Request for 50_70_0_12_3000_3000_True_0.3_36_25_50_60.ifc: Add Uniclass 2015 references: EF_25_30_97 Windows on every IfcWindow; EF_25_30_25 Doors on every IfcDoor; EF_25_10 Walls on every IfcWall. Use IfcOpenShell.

First a look at what the model holds.

```python
import ifcopenshell

model = ifcopenshell.open("50_70_0_12_3000_3000_True_0.3_36_25_50_60.ifc")
print(model.schema)
print("classifications:", [c.Name for c in model.by_type("IfcClassification")])
for ifc_class in ("IfcDoor", "IfcRoof", "IfcStair", "IfcWall", "IfcWindow"):
    print(ifc_class, len(model.by_type(ifc_class)))
```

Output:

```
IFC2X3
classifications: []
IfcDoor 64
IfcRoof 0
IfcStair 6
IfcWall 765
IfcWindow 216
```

```python
import ifcopenshell
import ifcopenshell.api.classification

model = ifcopenshell.open("50_70_0_12_3000_3000_True_0.3_36_25_50_60.ifc")

# IFC2X3 requires Source and Edition and has no link from the project to the system.
system = model.create_entity("IfcClassification", Source="NBS", Edition="2015", Name="Uniclass 2015")

codes = {
    "IfcWindow": ("EF_25_30_97", "Windows"),
    "IfcDoor": ("EF_25_30_25", "Doors"),
    "IfcWall": ("EF_25_10", "Walls"),
}
for ifc_class, (code, name) in codes.items():
    products = model.by_type(ifc_class)
    ifcopenshell.api.classification.add_reference(
        model, products=products, classification=system, identification=code, name=name
    )
    print(code, len(products))

model.write("50_70_0_12_3000_3000_True_0.3_36_25_50_60_edited.ifc")
```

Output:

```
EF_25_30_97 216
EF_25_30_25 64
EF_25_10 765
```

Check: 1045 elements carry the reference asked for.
